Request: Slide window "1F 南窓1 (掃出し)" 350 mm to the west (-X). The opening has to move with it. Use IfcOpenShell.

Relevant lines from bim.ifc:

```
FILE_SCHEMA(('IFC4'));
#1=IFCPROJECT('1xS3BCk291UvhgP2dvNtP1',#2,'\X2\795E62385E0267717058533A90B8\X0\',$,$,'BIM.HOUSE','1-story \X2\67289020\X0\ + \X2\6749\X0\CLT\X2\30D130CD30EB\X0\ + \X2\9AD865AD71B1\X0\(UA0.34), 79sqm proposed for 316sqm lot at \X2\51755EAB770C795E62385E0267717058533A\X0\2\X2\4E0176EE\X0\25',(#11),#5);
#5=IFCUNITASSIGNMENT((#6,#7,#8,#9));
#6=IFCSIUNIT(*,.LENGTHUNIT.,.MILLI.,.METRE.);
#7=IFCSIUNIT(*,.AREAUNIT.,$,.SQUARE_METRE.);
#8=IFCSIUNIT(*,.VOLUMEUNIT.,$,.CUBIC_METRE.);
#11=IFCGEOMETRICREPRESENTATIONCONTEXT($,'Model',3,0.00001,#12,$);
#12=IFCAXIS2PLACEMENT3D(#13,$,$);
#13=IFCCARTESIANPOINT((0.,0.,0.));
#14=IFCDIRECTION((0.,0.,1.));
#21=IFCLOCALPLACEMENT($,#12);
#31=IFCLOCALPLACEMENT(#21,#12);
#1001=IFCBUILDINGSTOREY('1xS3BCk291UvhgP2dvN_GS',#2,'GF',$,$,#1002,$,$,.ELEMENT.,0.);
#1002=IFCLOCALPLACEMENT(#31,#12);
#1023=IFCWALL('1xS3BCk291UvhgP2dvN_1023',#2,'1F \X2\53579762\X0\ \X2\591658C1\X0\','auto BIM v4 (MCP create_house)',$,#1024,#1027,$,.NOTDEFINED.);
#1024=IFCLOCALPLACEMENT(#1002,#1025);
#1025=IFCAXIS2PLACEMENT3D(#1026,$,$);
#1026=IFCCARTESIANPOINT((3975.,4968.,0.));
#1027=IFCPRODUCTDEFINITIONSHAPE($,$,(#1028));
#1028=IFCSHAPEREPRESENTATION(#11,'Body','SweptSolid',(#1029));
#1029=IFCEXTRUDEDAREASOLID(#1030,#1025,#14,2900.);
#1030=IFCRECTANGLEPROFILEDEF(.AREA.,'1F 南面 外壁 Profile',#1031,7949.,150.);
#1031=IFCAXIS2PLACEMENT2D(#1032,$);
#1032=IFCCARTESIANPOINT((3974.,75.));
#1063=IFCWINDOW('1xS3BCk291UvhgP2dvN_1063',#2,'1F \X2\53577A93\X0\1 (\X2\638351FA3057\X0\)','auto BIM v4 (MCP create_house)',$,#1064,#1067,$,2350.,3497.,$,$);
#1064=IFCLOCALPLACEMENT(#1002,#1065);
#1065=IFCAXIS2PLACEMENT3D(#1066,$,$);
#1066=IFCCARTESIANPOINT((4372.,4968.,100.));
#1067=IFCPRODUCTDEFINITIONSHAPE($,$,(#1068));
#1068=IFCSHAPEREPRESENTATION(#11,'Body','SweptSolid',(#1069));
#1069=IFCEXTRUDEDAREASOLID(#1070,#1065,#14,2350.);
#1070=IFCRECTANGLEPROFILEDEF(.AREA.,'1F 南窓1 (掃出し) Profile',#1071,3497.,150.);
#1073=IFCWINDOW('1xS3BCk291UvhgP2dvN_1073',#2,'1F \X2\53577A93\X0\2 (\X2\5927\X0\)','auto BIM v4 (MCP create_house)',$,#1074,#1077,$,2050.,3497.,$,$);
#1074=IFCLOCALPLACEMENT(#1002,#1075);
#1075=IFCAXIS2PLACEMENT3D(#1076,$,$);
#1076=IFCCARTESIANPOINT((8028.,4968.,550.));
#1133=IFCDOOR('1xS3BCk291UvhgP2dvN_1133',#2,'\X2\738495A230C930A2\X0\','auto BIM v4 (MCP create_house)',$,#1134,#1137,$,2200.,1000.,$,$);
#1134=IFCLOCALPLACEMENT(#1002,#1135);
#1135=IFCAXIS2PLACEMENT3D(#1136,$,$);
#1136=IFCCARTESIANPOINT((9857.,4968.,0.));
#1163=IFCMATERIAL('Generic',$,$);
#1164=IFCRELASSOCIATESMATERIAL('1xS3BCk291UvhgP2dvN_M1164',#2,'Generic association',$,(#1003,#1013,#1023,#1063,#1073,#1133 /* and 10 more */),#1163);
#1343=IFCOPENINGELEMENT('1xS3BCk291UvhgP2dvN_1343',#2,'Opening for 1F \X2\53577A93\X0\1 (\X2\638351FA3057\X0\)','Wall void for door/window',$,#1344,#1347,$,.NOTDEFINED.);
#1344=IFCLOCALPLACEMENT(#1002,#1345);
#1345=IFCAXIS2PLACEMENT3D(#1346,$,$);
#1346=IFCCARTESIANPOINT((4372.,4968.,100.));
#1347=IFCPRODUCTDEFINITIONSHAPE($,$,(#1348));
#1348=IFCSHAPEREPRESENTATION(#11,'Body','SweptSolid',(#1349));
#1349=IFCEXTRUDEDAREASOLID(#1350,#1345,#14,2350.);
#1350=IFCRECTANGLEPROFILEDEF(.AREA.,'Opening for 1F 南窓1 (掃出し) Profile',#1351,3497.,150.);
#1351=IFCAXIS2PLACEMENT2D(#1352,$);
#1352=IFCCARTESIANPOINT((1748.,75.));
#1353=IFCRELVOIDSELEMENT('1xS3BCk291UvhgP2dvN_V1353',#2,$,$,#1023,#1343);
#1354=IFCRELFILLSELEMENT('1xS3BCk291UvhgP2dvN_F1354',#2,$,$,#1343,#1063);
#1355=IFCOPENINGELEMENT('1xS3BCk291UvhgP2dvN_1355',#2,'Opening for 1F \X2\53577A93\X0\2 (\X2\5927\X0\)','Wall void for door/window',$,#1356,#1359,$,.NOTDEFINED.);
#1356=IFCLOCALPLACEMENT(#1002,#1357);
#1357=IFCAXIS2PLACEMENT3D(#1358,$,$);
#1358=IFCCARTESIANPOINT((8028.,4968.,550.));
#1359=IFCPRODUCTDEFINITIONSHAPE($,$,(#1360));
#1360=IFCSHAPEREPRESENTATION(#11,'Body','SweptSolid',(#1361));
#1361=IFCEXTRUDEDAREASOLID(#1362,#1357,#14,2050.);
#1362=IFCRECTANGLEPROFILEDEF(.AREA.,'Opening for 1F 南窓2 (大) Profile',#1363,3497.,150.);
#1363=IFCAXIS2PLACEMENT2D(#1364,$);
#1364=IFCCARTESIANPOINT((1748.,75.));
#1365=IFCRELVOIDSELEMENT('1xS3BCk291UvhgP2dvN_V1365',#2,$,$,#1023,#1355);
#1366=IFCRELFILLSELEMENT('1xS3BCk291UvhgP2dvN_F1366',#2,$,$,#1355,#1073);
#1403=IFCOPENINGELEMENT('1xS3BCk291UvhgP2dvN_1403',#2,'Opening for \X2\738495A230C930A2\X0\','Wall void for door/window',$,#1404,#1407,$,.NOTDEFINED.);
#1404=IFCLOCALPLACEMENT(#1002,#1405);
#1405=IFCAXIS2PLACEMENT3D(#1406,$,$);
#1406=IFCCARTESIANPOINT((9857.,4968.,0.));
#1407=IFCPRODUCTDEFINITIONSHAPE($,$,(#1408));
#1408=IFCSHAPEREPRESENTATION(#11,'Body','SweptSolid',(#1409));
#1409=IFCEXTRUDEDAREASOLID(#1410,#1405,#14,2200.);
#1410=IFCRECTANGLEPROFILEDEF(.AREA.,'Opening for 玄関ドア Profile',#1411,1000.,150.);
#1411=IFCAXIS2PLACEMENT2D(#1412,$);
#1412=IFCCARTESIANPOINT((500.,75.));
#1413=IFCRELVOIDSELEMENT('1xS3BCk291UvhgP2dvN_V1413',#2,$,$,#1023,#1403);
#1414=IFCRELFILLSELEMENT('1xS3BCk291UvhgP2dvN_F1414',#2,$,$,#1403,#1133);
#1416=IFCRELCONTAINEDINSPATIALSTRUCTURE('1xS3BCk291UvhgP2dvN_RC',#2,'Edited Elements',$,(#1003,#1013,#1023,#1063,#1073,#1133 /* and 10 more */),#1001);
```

```python
import ifcopenshell
import ifcopenshell.api.geometry
import ifcopenshell.util.placement
import ifcopenshell.util.unit

model = ifcopenshell.open("bim.ifc")
unit_scale = ifcopenshell.util.unit.calculate_unit_scale(model)

window = model.by_guid("1xS3BCk291UvhgP2dvN_1063")
opening = window.FillsVoids[0].RelatingOpeningElement
wall = opening.VoidsElements[0].RelatingBuildingElement

wall_matrix = ifcopenshell.util.placement.get_local_placement(wall.ObjectPlacement)
shift = wall_matrix[:3, 0] * -0.35 / unit_scale
before = ifcopenshell.util.placement.get_local_placement(window.ObjectPlacement)[:3, 3].copy()

# The window is not placed relative to its opening, so move both.
for product in (opening, window):
    matrix = ifcopenshell.util.placement.get_local_placement(product.ObjectPlacement)
    matrix[:3, 3] += shift
    ifcopenshell.api.geometry.edit_object_placement(model, product=product, matrix=matrix, is_si=False)

after = ifcopenshell.util.placement.get_local_placement(window.ObjectPlacement)[:3, 3]
print("window moved by", (after - before).round(3) + 0.0)

model.write("bim_rev.ifc")
```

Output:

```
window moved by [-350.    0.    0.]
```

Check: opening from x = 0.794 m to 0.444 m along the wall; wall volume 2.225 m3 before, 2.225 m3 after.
